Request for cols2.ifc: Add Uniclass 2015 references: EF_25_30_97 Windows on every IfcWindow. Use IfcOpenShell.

First a look at what the model holds.

```python
import ifcopenshell

model = ifcopenshell.open("cols2.ifc")
print(model.schema)
print("classifications:", [c.Name for c in model.by_type("IfcClassification")])
for ifc_class in ("IfcDoor", "IfcRoof", "IfcStair", "IfcWall", "IfcWindow"):
    print(ifc_class, len(model.by_type(ifc_class)))
```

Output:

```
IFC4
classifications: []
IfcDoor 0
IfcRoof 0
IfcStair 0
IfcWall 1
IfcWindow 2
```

```python
import ifcopenshell
import ifcopenshell.api.classification

model = ifcopenshell.open("cols2.ifc")

system = ifcopenshell.api.classification.add_classification(model, classification="Uniclass 2015")

codes = {
    "IfcWindow": ("EF_25_30_97", "Windows"),
}
for ifc_class, (code, name) in codes.items():
    products = model.by_type(ifc_class)
    ifcopenshell.api.classification.add_reference(
        model, products=products, classification=system, identification=code, name=name
    )
    print(code, len(products))

model.write("cols2_edited.ifc")
```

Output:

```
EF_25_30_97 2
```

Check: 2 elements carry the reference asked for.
